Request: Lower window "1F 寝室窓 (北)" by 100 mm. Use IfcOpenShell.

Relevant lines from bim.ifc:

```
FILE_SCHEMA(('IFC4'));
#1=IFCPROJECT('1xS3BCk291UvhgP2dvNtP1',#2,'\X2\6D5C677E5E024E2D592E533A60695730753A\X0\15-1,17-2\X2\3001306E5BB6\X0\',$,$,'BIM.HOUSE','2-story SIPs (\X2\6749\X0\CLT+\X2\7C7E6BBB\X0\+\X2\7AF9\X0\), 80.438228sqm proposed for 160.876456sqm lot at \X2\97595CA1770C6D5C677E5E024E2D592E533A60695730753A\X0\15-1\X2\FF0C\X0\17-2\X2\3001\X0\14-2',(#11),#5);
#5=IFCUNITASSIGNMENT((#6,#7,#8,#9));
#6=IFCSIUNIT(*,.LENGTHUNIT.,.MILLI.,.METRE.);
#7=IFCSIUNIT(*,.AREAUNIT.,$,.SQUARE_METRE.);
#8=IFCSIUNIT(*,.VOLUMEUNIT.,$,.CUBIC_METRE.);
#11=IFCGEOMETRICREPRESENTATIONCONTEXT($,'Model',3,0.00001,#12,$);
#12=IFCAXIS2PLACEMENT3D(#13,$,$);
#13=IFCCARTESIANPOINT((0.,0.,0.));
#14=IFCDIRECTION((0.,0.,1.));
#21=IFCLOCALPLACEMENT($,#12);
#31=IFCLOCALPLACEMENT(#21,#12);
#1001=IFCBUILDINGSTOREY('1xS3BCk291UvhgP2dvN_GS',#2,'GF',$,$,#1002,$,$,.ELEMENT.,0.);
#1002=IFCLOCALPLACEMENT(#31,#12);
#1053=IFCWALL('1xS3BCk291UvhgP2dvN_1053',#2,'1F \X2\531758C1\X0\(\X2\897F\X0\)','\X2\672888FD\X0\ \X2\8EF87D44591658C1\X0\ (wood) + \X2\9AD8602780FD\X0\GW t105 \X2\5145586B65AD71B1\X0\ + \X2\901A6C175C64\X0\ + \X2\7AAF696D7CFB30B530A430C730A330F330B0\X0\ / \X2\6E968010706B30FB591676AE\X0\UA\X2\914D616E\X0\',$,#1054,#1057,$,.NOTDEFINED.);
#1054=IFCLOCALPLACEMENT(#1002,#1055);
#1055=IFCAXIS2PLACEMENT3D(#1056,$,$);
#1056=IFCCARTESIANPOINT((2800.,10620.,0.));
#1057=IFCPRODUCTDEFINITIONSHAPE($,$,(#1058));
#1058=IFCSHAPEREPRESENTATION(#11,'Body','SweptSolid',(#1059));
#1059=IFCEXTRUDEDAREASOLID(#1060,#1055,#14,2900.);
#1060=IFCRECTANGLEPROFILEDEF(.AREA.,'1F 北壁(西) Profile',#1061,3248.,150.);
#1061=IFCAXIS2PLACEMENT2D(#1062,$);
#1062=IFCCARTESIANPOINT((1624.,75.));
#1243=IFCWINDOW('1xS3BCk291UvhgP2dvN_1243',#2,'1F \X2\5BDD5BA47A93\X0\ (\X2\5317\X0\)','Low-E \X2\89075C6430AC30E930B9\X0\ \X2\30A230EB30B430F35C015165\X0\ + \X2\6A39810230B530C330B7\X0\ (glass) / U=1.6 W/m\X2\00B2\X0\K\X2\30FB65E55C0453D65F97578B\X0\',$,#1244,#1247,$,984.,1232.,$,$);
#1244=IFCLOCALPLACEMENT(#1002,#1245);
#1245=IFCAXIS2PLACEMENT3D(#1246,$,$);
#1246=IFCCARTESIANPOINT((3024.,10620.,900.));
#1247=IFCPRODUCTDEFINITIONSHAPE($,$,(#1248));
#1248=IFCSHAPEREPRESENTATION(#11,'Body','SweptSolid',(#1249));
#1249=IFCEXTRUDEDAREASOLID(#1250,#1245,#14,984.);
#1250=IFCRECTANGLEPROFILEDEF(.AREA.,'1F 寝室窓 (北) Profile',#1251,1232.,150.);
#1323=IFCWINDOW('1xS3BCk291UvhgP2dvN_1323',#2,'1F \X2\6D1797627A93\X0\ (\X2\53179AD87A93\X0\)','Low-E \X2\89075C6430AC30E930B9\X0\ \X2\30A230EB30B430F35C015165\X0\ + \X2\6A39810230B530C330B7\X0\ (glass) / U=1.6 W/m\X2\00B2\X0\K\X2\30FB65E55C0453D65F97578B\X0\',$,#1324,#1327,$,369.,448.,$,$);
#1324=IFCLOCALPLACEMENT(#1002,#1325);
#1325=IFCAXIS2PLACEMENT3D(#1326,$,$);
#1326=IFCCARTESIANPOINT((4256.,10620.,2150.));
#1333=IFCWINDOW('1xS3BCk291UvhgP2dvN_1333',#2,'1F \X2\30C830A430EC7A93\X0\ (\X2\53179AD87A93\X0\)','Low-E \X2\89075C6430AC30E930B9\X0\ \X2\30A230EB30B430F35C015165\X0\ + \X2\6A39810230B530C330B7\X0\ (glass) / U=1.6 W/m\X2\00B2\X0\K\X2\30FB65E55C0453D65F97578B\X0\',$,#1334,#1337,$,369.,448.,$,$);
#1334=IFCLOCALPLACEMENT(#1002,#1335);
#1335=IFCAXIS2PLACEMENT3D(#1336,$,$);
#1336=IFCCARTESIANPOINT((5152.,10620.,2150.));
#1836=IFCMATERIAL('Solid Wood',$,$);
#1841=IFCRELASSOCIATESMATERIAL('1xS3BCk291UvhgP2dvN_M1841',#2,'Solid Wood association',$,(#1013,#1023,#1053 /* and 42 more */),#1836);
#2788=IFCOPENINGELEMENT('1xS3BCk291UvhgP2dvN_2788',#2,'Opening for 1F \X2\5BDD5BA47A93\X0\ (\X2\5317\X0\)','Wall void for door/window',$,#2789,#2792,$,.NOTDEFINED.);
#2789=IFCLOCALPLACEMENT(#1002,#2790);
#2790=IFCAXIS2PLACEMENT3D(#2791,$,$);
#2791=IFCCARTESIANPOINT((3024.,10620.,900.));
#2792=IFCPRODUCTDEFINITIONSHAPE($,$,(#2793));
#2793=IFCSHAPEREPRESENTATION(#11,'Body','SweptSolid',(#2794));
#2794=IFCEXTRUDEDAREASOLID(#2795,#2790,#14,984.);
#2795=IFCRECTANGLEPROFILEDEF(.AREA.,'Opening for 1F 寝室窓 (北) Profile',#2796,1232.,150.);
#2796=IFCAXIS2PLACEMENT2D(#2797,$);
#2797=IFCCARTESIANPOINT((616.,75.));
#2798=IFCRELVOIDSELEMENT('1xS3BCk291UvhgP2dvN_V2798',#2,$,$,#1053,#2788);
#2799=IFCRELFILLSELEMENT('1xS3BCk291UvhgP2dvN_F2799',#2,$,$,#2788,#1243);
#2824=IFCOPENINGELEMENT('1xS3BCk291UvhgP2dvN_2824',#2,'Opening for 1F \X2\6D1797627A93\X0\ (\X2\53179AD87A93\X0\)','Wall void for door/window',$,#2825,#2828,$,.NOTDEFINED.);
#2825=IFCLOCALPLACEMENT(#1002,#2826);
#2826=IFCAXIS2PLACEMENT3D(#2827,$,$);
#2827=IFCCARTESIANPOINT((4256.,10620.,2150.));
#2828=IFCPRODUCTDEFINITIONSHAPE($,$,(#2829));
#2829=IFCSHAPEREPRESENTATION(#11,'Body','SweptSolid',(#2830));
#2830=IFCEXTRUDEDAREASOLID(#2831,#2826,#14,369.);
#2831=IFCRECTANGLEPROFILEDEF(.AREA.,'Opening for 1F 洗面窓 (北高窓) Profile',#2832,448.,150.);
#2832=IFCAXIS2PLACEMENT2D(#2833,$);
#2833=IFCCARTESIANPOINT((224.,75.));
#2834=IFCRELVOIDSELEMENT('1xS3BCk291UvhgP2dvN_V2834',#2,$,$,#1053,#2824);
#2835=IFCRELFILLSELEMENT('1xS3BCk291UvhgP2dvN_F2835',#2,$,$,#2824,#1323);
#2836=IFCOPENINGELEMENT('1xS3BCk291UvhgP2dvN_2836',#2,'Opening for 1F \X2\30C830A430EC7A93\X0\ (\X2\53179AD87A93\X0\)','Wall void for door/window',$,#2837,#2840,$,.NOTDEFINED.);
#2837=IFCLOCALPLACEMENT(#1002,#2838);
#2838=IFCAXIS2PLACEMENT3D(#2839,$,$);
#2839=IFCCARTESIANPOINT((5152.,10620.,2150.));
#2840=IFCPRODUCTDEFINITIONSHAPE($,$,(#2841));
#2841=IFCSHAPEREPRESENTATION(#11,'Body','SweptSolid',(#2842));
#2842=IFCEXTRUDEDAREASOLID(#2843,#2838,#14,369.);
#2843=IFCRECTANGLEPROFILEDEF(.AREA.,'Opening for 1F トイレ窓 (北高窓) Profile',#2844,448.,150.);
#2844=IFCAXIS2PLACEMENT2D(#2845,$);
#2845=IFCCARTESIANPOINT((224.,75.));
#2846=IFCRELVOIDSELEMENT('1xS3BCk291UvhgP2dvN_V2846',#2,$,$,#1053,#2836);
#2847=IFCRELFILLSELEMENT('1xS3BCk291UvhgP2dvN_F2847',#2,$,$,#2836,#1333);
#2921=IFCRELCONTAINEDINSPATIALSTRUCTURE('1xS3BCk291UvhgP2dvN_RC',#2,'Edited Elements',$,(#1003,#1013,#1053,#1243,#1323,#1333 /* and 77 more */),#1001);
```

```python
import numpy as np
import ifcopenshell
import ifcopenshell.api.geometry
import ifcopenshell.util.placement
import ifcopenshell.util.unit

model = ifcopenshell.open("bim.ifc")
unit_scale = ifcopenshell.util.unit.calculate_unit_scale(model)

window = model.by_guid("1xS3BCk291UvhgP2dvN_1243")
opening = window.FillsVoids[0].RelatingOpeningElement
dz = -100.0

shift = np.array([0.0, 0.0, dz])
# The window is not placed relative to its opening, so move both.
for product in (opening, window):
    matrix = ifcopenshell.util.placement.get_local_placement(product.ObjectPlacement)
    matrix[:3, 3] += shift
    ifcopenshell.api.geometry.edit_object_placement(model, product=product, matrix=matrix, is_si=False)

print(f"moved by {dz * unit_scale:+.3f} m")

model.write("bim_rev.ifc")
```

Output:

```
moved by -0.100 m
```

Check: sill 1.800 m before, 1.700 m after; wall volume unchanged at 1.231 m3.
